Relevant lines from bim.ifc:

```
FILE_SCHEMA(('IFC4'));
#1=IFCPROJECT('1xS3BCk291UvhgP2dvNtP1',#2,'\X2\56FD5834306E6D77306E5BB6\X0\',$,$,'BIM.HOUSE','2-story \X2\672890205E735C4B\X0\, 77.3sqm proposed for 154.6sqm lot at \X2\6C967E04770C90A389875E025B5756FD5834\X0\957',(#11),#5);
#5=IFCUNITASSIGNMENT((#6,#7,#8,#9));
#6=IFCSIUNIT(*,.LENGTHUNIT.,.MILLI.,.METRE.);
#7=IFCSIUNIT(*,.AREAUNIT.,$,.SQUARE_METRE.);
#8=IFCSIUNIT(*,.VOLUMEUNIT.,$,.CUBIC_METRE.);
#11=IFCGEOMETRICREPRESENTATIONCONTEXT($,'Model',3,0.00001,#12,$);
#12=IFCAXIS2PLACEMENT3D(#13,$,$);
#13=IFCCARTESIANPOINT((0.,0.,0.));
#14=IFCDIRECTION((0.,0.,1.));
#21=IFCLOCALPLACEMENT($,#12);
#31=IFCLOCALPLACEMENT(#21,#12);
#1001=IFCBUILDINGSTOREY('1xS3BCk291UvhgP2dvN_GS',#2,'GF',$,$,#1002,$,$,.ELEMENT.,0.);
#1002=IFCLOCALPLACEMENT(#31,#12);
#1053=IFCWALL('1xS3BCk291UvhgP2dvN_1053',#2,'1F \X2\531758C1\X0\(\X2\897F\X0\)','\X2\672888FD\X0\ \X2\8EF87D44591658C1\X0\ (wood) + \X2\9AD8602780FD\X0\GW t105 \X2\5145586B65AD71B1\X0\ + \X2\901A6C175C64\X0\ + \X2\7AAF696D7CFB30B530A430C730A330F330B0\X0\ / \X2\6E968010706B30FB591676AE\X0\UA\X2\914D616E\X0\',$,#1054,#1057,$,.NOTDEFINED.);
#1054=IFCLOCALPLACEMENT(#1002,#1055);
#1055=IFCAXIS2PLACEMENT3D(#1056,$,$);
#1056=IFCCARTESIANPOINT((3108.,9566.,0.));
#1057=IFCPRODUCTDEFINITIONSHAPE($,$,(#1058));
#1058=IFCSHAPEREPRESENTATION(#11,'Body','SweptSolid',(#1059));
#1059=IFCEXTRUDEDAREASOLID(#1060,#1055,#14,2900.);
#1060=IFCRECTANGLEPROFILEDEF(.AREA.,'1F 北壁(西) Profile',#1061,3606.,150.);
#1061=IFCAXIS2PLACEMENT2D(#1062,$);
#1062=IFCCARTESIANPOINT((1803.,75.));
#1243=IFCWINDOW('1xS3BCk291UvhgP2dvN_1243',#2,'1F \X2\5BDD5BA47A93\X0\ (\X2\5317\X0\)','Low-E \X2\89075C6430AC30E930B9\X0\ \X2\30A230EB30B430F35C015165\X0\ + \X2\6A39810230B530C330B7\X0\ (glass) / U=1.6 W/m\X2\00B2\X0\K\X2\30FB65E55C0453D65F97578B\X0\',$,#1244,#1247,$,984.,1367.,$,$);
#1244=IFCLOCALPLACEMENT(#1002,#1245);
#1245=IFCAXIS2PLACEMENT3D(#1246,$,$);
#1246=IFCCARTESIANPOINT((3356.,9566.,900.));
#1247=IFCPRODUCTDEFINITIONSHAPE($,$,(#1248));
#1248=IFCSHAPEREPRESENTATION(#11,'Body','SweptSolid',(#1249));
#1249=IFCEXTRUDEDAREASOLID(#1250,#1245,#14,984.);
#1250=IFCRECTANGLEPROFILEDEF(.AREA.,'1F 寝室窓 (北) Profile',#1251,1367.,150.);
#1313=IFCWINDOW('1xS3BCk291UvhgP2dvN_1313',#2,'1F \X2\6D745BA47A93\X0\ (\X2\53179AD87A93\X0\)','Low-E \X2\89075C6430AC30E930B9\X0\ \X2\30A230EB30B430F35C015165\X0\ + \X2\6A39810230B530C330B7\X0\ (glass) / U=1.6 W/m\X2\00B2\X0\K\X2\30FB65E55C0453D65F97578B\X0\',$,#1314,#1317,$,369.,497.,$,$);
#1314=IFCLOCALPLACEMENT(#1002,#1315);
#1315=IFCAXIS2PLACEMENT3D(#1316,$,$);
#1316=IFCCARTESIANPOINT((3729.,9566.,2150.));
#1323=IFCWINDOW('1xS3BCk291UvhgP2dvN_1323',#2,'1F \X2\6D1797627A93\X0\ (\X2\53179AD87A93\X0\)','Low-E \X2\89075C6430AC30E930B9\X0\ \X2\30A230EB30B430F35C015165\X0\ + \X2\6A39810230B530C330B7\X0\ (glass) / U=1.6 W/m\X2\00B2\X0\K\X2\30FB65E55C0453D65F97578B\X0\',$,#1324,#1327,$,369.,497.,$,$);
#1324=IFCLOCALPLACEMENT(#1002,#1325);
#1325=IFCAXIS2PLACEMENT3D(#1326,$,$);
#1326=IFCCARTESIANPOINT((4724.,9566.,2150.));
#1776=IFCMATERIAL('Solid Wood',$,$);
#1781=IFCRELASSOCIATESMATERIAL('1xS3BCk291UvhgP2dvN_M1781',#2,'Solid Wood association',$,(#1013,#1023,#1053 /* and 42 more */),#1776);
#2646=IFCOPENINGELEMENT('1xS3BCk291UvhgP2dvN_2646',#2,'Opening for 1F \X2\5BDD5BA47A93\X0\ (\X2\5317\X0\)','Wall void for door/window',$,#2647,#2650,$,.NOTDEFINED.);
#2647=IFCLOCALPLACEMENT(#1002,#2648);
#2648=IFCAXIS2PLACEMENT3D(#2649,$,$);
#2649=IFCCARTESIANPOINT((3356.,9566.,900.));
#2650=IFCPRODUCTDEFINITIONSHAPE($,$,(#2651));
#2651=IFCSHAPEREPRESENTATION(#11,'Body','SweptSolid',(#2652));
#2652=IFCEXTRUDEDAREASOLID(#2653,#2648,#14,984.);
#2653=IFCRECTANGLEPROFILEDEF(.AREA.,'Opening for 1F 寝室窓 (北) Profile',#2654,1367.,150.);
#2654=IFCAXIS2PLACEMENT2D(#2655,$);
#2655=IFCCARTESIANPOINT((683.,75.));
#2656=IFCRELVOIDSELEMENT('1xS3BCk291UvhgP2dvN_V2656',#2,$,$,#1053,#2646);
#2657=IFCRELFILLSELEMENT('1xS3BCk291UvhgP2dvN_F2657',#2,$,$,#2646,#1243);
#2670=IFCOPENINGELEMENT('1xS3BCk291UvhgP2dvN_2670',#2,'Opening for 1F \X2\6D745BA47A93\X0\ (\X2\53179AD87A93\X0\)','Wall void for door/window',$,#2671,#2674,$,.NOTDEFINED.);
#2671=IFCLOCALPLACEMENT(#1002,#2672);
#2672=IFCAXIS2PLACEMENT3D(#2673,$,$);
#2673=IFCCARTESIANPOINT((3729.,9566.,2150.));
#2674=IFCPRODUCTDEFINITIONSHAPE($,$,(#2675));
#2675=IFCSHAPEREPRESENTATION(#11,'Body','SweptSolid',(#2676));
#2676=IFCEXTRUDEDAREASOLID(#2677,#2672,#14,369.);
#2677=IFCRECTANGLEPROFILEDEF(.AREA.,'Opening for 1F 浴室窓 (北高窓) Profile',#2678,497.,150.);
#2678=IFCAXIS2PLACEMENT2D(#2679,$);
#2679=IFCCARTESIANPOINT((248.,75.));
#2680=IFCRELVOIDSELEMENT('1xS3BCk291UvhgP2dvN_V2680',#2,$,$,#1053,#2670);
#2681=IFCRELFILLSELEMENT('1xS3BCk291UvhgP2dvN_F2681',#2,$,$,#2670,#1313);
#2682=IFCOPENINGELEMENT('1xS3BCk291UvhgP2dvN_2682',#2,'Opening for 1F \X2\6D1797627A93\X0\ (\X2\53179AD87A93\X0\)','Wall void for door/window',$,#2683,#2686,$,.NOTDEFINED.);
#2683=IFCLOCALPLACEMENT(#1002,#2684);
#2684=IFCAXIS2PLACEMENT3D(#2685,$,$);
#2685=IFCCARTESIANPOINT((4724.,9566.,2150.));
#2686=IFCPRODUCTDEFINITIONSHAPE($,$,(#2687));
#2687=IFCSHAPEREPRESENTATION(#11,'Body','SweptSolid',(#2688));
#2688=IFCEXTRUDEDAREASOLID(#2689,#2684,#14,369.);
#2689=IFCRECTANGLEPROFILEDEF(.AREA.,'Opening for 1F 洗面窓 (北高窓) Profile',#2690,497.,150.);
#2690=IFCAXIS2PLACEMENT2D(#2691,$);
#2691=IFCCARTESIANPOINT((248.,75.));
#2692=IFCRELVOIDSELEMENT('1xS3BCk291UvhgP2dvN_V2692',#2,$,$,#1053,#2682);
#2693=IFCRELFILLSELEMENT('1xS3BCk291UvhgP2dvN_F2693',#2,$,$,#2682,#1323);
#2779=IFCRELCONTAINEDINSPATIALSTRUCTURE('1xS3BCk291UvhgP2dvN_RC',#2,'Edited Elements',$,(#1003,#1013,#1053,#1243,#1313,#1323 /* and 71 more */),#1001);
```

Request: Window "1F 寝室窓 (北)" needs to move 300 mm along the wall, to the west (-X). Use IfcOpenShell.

```python
import ifcopenshell
import ifcopenshell.api.geometry
import ifcopenshell.util.placement
import ifcopenshell.util.unit

model = ifcopenshell.open("bim.ifc")
unit_scale = ifcopenshell.util.unit.calculate_unit_scale(model)

window = model.by_id(1243)
opening = window.FillsVoids[0].RelatingOpeningElement
wall = opening.VoidsElements[0].RelatingBuildingElement

wall_matrix = ifcopenshell.util.placement.get_local_placement(wall.ObjectPlacement)
shift = wall_matrix[:3, 0] * -0.3 / unit_scale
before = ifcopenshell.util.placement.get_local_placement(window.ObjectPlacement)[:3, 3].copy()

# The window is not placed relative to its opening, so move both.
for product in (opening, window):
    matrix = ifcopenshell.util.placement.get_local_placement(product.ObjectPlacement)
    matrix[:3, 3] += shift
    ifcopenshell.api.geometry.edit_object_placement(model, product=product, matrix=matrix, is_si=False)

after = ifcopenshell.util.placement.get_local_placement(window.ObjectPlacement)[:3, 3]
print("window moved by", (after - before).round(3) + 0.0)

model.write("bim_edited.ifc")
```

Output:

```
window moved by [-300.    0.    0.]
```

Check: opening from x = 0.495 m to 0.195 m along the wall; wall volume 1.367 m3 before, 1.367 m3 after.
